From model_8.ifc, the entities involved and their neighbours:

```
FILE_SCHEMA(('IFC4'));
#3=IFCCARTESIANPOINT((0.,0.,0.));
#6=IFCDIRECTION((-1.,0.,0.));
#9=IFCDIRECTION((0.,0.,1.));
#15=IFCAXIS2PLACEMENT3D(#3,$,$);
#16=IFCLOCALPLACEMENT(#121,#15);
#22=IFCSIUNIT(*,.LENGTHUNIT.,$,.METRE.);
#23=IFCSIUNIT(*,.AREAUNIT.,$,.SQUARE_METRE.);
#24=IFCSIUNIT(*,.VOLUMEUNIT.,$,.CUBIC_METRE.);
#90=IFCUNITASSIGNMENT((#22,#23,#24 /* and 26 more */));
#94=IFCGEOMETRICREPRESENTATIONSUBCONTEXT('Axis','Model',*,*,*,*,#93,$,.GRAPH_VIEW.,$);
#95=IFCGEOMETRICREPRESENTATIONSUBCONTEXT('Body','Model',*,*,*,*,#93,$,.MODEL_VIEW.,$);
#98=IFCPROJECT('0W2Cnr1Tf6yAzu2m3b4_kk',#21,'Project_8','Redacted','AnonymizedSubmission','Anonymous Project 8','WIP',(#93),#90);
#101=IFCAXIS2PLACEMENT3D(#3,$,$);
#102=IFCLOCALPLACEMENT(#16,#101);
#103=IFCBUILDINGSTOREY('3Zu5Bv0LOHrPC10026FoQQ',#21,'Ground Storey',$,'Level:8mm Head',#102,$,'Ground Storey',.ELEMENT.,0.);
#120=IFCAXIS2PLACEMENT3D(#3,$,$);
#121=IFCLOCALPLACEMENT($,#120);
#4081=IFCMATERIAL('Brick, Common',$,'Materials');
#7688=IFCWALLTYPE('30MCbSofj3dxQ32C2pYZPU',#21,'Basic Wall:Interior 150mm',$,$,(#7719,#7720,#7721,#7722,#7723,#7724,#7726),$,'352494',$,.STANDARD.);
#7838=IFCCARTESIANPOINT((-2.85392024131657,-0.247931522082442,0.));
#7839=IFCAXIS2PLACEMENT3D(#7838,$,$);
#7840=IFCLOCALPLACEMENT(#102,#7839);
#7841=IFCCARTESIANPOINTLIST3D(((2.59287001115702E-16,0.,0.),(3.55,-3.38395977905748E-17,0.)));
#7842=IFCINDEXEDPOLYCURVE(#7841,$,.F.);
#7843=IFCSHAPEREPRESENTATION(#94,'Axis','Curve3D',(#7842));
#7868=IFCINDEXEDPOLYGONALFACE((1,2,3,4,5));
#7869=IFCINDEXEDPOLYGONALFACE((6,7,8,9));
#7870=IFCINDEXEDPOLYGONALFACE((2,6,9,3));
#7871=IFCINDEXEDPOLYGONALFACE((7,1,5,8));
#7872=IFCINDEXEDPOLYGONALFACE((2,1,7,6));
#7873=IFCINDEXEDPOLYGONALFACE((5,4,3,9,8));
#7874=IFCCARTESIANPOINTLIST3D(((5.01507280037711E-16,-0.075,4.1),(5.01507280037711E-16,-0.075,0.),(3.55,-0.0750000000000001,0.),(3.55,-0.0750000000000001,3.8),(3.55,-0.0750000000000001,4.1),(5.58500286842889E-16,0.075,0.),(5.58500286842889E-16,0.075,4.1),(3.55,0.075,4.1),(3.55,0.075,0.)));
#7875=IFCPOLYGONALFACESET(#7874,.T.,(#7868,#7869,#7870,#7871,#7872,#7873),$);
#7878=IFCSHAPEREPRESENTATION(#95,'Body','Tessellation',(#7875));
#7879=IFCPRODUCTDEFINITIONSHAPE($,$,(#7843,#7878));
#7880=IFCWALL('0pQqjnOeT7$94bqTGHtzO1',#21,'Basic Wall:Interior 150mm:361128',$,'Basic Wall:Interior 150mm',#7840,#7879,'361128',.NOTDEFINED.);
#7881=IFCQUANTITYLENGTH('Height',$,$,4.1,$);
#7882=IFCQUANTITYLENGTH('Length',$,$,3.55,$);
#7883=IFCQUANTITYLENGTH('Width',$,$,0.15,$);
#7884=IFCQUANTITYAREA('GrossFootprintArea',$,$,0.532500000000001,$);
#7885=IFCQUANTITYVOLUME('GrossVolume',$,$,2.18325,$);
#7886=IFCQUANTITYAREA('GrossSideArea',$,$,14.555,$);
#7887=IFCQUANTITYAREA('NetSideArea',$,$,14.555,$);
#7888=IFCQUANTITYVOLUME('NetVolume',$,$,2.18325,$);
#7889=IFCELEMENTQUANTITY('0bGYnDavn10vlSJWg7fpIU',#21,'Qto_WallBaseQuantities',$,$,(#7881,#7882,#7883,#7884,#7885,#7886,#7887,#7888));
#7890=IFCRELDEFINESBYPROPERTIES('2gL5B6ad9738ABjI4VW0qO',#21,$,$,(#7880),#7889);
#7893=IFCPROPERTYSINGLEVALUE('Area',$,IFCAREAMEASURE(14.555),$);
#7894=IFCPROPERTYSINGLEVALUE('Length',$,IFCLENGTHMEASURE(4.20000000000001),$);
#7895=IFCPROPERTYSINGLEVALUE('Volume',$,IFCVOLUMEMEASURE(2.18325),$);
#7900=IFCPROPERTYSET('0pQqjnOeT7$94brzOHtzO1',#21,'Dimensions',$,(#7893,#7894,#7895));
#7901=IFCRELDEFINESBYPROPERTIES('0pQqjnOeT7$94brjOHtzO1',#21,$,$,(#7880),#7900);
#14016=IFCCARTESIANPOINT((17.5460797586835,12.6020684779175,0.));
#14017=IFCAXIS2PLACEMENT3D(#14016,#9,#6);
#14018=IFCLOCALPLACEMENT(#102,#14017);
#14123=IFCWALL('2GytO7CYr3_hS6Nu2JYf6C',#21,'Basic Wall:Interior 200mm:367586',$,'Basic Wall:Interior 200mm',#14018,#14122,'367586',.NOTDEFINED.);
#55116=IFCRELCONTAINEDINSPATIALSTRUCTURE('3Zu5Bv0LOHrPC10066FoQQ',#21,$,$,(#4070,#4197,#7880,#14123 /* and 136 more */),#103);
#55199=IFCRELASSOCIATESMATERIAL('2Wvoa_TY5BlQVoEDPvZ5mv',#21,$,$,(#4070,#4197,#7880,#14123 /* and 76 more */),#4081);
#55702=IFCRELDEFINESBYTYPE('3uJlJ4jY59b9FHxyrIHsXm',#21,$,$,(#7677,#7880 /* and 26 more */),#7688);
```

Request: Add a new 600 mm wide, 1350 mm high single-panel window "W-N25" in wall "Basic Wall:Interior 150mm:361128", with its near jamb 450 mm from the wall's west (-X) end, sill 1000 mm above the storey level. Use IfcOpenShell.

```python
import numpy as np
import ifcopenshell
import ifcopenshell.api.feature
import ifcopenshell.api.geometry
import ifcopenshell.api.pset
import ifcopenshell.api.root
import ifcopenshell.api.spatial
import ifcopenshell.geom
import ifcopenshell.util.element
import ifcopenshell.util.placement
import ifcopenshell.util.representation
import ifcopenshell.util.shape
import ifcopenshell.util.unit

model = ifcopenshell.open("model_8.ifc")
unit_scale = ifcopenshell.util.unit.calculate_unit_scale(model)
area_scale = ifcopenshell.util.unit.calculate_unit_scale(model, "AREAUNIT")
volume_scale = ifcopenshell.util.unit.calculate_unit_scale(model, "VOLUMEUNIT")
settings = ifcopenshell.geom.settings()


def volume(element):
    """Net volume in cubic metres, openings subtracted."""
    shape = ifcopenshell.geom.create_shape(settings, element)
    return ifcopenshell.util.shape.get_volume(shape.geometry)


wall = model.by_guid("0pQqjnOeT7$94bqTGHtzO1")
storey = ifcopenshell.util.element.get_container(wall, ifc_class="IfcBuildingStorey")
context = ifcopenshell.util.representation.get_context(model, "Model", "Body", "MODEL_VIEW")
before = volume(wall)

width, height, from_end, sill = 0.6, 1.35, 0.45, 1  # metres

# The wall runs along its own X axis, and the end named is its -X end.
wall_shape = ifcopenshell.geom.create_shape(settings, wall)
x, y, z = ifcopenshell.util.shape.get_vertices(wall_shape.geometry).T
start = x.min() + from_end
face, thickness = float(y.min()), float(y.max() - y.min())
wall_matrix = ifcopenshell.util.placement.get_local_placement(wall.ObjectPlacement)
level = ifcopenshell.util.placement.get_local_placement(storey.ObjectPlacement)[2, 3]


def in_wall(x, y):
    """Placement at x, y metres in the wall's axes, at sill height."""
    matrix = wall_matrix.copy()
    matrix[:, 3] = wall_matrix @ np.array([x / unit_scale, y / unit_scale, 0.0, 1.0])
    matrix[2, 3] = level + sill / unit_scale
    return matrix


# Opening: a box that overshoots both wall faces by 50 mm.
opening = ifcopenshell.api.root.create_entity(model, ifc_class="IfcOpeningElement", predefined_type="OPENING")
box = ifcopenshell.api.geometry.add_wall_representation(
    model, context=context, length=width, height=height, thickness=thickness + 0.1
)
ifcopenshell.api.geometry.assign_representation(model, product=opening, representation=box)
ifcopenshell.api.geometry.edit_object_placement(model, product=opening, matrix=in_wall(start, face - 0.05), is_si=False)
ifcopenshell.api.feature.add_feature(model, feature=opening, element=wall)

window = ifcopenshell.api.root.create_entity(model, ifc_class="IfcWindow", name="W-N25", predefined_type="WINDOW")
window.OverallWidth, window.OverallHeight = width / unit_scale, height / unit_scale
window.PartitioningType = "SINGLE_PANEL"
body = ifcopenshell.api.geometry.add_window_representation(
    model,
    context=context,
    overall_width=window.OverallWidth,
    overall_height=window.OverallHeight,
    partition_type="SINGLE_PANEL",
)
ifcopenshell.api.geometry.assign_representation(model, product=window, representation=body)
ifcopenshell.api.spatial.assign_container(model, products=[window], relating_structure=storey)
ifcopenshell.api.feature.add_filling(model, opening=opening, element=window)

# Centre the window in the wall's thickness.
ifcopenshell.api.geometry.edit_object_placement(model, product=window, matrix=in_wall(start, face), is_si=False)
window_shape = ifcopenshell.geom.create_shape(settings, window)
depth = ifcopenshell.util.shape.get_vertices(window_shape.geometry)[:, 1]
offset = face + thickness / 2 - (depth.min() + depth.max()) / 2
ifcopenshell.api.geometry.edit_object_placement(model, product=window, matrix=in_wall(start, offset), is_si=False)

after = volume(wall)

# Update the wall's stored quantities.
qto = model.by_id(ifcopenshell.util.element.get_pset(wall, "Qto_WallBaseQuantities", should_inherit=False)["id"])
ifcopenshell.api.pset.edit_qto(model, qto=qto, properties={
    "NetSideArea": after / thickness / area_scale,
    "NetVolume": after / volume_scale,
})
pset = model.by_id(ifcopenshell.util.element.get_pset(wall, "Dimensions", should_inherit=False)["id"])
ifcopenshell.api.pset.edit_pset(model, pset=pset, properties={
    "Area": model.create_entity("IfcAreaMeasure", after / thickness / area_scale),
    "Volume": model.create_entity("IfcVolumeMeasure", after / volume_scale),
})

print(f"wall volume {before:.3f} -> {after:.3f} m3")

model.write("model_8-out.ifc")
```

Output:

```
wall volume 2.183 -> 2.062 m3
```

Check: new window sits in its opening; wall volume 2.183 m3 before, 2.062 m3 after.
